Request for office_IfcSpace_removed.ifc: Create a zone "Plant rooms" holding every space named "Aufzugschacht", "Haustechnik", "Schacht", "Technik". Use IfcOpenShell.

First a look at what the model holds.

```python
import ifcopenshell

model = ifcopenshell.open("office_IfcSpace_removed.ifc")
print(model.schema)
seen = {}
for space in model.by_type("IfcSpace"):
    seen[space.LongName] = seen.get(space.LongName, 0) + 1
for name, count in sorted(seen.items(), key=str):
    print(count, "x", name)
print("zones:", [z.Name for z in model.by_type("IfcZone")][:20])
```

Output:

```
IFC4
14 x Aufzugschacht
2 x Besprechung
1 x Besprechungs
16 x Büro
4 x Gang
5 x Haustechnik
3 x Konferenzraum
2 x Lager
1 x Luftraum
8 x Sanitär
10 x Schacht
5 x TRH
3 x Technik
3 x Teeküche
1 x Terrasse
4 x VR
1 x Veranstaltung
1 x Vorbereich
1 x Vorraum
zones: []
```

```python
import ifcopenshell
import ifcopenshell.api.group
import ifcopenshell.api.root

model = ifcopenshell.open("office_IfcSpace_removed.ifc")

names = {"Aufzugschacht", "Haustechnik", "Schacht", "Technik"}
spaces = [s for s in model.by_type("IfcSpace") if s.LongName in names]

zone = ifcopenshell.api.root.create_entity(model, ifc_class="IfcZone", name="Plant rooms")
ifcopenshell.api.group.assign_group(model, products=spaces, group=zone)
print(len(spaces), "spaces in", zone.Name)

model.write("office_IfcSpace_removed_edited.ifc")
```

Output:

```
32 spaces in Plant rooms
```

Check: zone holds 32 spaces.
